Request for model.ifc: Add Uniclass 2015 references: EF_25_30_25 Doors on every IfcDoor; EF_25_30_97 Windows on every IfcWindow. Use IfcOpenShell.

First a look at what the model holds.

```python
import ifcopenshell

model = ifcopenshell.open("model.ifc")
print(model.schema)
print("classifications:", [c.Name for c in model.by_type("IfcClassification")])
for ifc_class in ("IfcDoor", "IfcRoof", "IfcStair", "IfcWall", "IfcWindow"):
    print(ifc_class, len(model.by_type(ifc_class)))
```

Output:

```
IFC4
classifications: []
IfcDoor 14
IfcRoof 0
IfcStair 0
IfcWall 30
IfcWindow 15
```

```python
import ifcopenshell
import ifcopenshell.api.classification

model = ifcopenshell.open("model.ifc")

system = ifcopenshell.api.classification.add_classification(model, classification="Uniclass 2015")

codes = {
    "IfcDoor": ("EF_25_30_25", "Doors"),
    "IfcWindow": ("EF_25_30_97", "Windows"),
}
for ifc_class, (code, name) in codes.items():
    products = model.by_type(ifc_class)
    ifcopenshell.api.classification.add_reference(
        model, products=products, classification=system, identification=code, name=name
    )
    print(code, len(products))

model.write("model-out.ifc")
```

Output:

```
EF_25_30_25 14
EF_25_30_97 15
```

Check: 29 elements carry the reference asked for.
